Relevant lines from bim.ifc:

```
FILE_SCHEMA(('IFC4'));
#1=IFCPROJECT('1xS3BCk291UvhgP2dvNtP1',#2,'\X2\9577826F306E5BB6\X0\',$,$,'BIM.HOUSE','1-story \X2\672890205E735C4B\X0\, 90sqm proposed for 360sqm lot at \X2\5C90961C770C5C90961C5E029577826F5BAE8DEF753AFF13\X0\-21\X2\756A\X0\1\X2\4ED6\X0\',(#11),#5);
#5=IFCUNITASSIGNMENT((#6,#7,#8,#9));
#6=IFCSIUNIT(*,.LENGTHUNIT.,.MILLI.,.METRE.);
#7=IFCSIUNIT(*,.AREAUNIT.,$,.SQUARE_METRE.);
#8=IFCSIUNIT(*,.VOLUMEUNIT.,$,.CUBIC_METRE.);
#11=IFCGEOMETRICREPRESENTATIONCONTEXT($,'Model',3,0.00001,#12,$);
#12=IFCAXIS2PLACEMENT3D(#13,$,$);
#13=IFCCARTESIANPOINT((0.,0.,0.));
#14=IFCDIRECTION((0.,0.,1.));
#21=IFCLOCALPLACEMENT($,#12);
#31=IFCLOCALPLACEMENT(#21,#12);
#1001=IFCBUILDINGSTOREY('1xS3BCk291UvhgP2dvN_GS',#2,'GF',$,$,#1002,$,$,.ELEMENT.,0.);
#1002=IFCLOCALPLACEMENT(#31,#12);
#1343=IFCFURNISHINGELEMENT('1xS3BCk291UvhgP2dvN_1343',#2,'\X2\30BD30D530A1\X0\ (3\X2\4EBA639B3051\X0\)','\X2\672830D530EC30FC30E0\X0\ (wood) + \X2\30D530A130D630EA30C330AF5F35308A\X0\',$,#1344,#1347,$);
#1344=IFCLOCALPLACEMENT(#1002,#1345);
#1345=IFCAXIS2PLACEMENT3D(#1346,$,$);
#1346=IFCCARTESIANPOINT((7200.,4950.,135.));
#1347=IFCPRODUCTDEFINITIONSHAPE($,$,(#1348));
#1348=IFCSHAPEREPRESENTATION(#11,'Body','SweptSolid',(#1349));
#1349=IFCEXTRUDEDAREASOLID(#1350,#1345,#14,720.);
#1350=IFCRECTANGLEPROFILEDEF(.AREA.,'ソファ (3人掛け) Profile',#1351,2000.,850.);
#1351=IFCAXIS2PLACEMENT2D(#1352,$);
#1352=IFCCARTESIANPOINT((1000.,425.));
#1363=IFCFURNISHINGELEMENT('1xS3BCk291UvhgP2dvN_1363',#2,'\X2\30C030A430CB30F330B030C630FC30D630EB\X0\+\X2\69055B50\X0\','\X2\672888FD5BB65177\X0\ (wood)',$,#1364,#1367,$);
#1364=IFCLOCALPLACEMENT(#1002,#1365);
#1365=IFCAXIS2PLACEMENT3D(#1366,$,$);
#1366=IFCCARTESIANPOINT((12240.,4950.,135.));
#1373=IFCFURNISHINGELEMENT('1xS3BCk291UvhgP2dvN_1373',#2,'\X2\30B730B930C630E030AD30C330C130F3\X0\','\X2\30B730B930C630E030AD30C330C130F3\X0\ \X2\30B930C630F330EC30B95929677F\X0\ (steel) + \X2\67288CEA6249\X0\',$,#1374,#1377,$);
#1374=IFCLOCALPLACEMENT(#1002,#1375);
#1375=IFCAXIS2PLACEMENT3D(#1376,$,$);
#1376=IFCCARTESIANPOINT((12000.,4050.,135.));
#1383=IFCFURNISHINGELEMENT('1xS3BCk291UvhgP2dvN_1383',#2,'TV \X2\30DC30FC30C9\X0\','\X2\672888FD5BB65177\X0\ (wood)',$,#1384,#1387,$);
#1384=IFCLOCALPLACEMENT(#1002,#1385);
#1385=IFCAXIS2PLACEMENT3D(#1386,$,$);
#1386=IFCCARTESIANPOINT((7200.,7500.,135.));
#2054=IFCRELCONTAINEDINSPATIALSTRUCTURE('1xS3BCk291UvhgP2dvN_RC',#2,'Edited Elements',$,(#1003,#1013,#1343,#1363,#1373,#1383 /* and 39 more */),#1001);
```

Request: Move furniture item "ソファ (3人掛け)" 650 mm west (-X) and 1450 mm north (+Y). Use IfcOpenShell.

```python
import ifcopenshell
import ifcopenshell.api.geometry
import ifcopenshell.util.placement

model = ifcopenshell.open("bim.ifc")

item = model.by_id(1343)
matrix = ifcopenshell.util.placement.get_local_placement(item.ObjectPlacement)
matrix[0, 3] -= 650.0
matrix[1, 3] += 1450.0
ifcopenshell.api.geometry.edit_object_placement(model, product=item, matrix=matrix, is_si=False)

print(ifcopenshell.util.placement.get_local_placement(item.ObjectPlacement).round(3) + 0.0)

model.write("bim-out.ifc")
```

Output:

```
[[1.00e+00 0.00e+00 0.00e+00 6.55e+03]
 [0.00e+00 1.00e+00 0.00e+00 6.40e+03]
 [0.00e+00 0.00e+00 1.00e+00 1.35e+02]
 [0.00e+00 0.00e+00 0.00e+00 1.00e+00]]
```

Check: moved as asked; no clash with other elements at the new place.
